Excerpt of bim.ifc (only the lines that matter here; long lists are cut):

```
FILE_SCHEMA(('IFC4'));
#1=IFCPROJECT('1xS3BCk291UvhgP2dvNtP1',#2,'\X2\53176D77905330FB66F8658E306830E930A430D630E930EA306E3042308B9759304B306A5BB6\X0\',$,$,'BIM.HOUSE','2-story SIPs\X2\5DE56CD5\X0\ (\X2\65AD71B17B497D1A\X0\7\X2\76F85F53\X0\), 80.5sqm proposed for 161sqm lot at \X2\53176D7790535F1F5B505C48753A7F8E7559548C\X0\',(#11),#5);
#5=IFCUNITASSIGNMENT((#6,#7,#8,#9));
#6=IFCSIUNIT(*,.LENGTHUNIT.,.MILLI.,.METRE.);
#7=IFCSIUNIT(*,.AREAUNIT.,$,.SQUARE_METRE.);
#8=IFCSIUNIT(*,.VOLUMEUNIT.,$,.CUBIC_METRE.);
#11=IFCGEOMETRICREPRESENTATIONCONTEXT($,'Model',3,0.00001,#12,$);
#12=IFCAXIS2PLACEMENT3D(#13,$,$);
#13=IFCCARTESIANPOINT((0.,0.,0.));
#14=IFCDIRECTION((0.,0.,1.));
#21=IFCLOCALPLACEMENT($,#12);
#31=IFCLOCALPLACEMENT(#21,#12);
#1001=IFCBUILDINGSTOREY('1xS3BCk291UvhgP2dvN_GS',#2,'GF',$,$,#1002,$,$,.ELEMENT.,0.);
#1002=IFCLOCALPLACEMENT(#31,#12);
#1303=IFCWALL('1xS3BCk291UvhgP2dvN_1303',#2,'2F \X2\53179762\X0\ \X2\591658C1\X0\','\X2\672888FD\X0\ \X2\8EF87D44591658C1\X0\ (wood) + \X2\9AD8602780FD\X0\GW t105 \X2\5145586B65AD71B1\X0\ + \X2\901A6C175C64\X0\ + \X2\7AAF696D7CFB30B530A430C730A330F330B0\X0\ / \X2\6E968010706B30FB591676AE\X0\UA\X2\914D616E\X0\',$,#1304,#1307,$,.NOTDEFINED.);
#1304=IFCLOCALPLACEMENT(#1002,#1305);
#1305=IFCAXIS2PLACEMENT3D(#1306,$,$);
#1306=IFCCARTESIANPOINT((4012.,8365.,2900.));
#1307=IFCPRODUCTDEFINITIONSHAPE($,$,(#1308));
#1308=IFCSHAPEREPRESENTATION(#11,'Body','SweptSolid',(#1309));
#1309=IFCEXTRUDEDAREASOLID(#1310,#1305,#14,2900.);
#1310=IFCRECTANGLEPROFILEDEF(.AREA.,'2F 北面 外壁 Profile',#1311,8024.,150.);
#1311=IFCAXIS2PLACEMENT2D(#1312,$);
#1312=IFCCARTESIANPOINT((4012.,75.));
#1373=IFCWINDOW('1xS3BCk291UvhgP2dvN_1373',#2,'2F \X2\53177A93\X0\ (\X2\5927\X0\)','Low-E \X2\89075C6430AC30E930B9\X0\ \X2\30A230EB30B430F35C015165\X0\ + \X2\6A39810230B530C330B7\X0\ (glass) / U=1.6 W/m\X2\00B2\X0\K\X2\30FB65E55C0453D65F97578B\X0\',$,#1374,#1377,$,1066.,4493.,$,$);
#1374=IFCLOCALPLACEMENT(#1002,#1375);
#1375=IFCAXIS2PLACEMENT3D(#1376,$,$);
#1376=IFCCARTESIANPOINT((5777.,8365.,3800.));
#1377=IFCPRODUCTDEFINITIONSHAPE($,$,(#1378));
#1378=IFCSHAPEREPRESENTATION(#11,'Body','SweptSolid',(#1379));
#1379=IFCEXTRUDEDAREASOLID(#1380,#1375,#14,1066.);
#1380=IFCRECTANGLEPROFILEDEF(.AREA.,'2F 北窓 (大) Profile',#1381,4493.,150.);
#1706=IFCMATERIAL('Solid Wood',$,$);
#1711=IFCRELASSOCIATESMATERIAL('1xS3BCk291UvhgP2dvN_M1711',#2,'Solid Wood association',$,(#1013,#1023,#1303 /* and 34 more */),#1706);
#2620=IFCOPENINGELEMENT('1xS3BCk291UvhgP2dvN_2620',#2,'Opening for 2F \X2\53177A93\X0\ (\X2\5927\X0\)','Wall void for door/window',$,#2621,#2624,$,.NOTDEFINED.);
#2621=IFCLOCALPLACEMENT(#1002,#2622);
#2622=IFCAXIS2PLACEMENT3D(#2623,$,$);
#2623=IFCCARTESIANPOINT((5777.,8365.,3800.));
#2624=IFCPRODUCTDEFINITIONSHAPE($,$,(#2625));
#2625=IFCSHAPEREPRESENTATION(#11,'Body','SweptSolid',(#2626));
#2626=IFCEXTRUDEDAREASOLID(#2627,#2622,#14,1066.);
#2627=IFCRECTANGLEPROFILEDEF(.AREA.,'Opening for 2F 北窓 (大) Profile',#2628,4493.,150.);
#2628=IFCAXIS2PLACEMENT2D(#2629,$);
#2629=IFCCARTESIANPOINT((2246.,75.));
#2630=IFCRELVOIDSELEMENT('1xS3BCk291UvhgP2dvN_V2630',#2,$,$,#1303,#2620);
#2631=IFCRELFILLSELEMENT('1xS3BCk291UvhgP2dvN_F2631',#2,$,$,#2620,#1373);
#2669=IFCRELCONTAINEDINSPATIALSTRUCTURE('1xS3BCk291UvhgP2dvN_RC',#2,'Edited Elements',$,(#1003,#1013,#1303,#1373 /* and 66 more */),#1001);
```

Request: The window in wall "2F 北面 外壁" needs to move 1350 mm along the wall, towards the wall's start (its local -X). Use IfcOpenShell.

```python
import ifcopenshell
import ifcopenshell.api.geometry
import ifcopenshell.util.placement
import ifcopenshell.util.unit

model = ifcopenshell.open("bim.ifc")
unit_scale = ifcopenshell.util.unit.calculate_unit_scale(model)

window = model.by_guid("1xS3BCk291UvhgP2dvN_1373")
opening = window.FillsVoids[0].RelatingOpeningElement
wall = opening.VoidsElements[0].RelatingBuildingElement

wall_matrix = ifcopenshell.util.placement.get_local_placement(wall.ObjectPlacement)
shift = wall_matrix[:3, 0] * -1.35 / unit_scale
before = ifcopenshell.util.placement.get_local_placement(window.ObjectPlacement)[:3, 3].copy()

# The window is not placed relative to its opening, so move both.
for product in (opening, window):
    matrix = ifcopenshell.util.placement.get_local_placement(product.ObjectPlacement)
    matrix[:3, 3] += shift
    ifcopenshell.api.geometry.edit_object_placement(model, product=product, matrix=matrix, is_si=False)

after = ifcopenshell.util.placement.get_local_placement(window.ObjectPlacement)[:3, 3]
print("window moved by", (after - before).round(3) + 0.0)

model.write("bim_rev.ifc")
```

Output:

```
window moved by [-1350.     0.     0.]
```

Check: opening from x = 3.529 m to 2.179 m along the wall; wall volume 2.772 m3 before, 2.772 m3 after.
